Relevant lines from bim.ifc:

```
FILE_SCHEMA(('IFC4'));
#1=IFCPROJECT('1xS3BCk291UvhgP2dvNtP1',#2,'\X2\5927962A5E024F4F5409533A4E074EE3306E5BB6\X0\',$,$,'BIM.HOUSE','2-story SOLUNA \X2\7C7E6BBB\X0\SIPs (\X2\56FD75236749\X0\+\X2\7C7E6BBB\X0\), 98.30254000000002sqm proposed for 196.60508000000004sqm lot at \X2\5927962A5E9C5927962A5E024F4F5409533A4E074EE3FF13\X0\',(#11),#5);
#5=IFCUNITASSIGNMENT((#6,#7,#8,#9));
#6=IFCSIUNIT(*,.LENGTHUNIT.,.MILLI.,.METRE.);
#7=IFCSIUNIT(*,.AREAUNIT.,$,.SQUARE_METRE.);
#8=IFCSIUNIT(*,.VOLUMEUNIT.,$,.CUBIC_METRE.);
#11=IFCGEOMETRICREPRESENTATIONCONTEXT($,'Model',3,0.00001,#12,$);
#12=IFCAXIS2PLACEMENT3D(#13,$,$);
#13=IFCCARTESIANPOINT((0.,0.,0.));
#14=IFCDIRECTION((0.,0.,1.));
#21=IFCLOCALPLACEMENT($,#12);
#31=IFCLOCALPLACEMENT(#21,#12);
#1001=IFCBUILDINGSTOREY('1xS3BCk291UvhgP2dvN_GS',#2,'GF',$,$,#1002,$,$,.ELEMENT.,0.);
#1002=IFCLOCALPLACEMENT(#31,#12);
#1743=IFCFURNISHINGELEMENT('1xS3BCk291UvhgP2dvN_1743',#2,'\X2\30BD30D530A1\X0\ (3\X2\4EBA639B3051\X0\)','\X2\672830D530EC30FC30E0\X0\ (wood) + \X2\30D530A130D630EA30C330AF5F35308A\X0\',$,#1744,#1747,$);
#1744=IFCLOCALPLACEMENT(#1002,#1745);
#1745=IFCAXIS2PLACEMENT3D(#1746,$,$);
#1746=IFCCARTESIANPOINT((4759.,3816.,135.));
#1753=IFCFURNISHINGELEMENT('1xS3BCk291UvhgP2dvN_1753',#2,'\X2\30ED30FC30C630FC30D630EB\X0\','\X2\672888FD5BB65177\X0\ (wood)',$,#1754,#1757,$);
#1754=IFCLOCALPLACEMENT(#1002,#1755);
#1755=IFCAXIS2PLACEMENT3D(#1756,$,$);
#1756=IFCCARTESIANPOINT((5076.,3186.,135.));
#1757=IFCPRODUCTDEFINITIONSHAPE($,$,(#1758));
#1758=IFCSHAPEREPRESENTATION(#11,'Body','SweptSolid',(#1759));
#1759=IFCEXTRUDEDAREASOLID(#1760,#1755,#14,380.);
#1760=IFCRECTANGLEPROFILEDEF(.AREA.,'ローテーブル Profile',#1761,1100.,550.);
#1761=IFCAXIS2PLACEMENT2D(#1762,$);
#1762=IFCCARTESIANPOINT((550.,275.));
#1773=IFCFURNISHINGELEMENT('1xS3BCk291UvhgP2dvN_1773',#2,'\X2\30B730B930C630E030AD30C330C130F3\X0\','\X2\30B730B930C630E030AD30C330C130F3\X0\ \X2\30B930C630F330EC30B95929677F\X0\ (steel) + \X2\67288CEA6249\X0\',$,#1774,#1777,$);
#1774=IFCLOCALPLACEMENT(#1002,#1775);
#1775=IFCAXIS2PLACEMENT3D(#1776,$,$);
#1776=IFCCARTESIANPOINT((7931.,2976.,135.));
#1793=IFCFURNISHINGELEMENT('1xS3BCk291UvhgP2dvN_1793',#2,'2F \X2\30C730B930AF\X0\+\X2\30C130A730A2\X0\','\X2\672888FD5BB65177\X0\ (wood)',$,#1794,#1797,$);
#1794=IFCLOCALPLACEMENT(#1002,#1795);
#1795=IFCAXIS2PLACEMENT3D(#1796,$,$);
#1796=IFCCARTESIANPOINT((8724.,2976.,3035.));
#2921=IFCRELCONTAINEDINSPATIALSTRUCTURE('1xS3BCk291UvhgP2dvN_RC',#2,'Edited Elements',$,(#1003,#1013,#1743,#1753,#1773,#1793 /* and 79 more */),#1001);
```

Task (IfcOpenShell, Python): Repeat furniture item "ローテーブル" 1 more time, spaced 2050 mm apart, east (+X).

```python
import numpy as np
import ifcopenshell
import ifcopenshell.api.geometry
import ifcopenshell.api.root
import ifcopenshell.util.element
import ifcopenshell.util.placement
import ifcopenshell.util.unit

model = ifcopenshell.open("bim.ifc")
unit_scale = ifcopenshell.util.unit.calculate_unit_scale(model)


def reuse_history(source, copy):
    """copy_class also copies each property set's owner history, people and application; keep the originals."""
    for rel in copy.IsDefinedBy:
        if rel.is_a("IfcRelDefinesByProperties") and (history := rel.RelatingPropertyDefinition.OwnerHistory):
            rel.RelatingPropertyDefinition.OwnerHistory = source.OwnerHistory
            ifcopenshell.util.element.remove_deep2(model, history)


source = model.by_guid("1xS3BCk291UvhgP2dvN_1753")
base = ifcopenshell.util.placement.get_local_placement(source.ObjectPlacement)
step = np.array([1.0, 0.0, 0.0]) * 2.05 / unit_scale

for i in range(1, 2):
    copy = ifcopenshell.api.root.copy_class(model, product=source)
    copy.Representation = ifcopenshell.util.element.copy_deep(
        model, source.Representation, exclude=["IfcGeometricRepresentationContext", "IfcRepresentationMap"]
    )
    reuse_history(source, copy)
    matrix = base.copy()
    matrix[:3, 3] += i * step
    print("added at", matrix[:3, 3].round(3) + 0.0)
    ifcopenshell.api.geometry.edit_object_placement(model, product=copy, matrix=matrix, is_si=False)

model.write("bim_v2.ifc")
```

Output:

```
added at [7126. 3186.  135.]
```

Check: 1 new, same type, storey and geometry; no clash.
